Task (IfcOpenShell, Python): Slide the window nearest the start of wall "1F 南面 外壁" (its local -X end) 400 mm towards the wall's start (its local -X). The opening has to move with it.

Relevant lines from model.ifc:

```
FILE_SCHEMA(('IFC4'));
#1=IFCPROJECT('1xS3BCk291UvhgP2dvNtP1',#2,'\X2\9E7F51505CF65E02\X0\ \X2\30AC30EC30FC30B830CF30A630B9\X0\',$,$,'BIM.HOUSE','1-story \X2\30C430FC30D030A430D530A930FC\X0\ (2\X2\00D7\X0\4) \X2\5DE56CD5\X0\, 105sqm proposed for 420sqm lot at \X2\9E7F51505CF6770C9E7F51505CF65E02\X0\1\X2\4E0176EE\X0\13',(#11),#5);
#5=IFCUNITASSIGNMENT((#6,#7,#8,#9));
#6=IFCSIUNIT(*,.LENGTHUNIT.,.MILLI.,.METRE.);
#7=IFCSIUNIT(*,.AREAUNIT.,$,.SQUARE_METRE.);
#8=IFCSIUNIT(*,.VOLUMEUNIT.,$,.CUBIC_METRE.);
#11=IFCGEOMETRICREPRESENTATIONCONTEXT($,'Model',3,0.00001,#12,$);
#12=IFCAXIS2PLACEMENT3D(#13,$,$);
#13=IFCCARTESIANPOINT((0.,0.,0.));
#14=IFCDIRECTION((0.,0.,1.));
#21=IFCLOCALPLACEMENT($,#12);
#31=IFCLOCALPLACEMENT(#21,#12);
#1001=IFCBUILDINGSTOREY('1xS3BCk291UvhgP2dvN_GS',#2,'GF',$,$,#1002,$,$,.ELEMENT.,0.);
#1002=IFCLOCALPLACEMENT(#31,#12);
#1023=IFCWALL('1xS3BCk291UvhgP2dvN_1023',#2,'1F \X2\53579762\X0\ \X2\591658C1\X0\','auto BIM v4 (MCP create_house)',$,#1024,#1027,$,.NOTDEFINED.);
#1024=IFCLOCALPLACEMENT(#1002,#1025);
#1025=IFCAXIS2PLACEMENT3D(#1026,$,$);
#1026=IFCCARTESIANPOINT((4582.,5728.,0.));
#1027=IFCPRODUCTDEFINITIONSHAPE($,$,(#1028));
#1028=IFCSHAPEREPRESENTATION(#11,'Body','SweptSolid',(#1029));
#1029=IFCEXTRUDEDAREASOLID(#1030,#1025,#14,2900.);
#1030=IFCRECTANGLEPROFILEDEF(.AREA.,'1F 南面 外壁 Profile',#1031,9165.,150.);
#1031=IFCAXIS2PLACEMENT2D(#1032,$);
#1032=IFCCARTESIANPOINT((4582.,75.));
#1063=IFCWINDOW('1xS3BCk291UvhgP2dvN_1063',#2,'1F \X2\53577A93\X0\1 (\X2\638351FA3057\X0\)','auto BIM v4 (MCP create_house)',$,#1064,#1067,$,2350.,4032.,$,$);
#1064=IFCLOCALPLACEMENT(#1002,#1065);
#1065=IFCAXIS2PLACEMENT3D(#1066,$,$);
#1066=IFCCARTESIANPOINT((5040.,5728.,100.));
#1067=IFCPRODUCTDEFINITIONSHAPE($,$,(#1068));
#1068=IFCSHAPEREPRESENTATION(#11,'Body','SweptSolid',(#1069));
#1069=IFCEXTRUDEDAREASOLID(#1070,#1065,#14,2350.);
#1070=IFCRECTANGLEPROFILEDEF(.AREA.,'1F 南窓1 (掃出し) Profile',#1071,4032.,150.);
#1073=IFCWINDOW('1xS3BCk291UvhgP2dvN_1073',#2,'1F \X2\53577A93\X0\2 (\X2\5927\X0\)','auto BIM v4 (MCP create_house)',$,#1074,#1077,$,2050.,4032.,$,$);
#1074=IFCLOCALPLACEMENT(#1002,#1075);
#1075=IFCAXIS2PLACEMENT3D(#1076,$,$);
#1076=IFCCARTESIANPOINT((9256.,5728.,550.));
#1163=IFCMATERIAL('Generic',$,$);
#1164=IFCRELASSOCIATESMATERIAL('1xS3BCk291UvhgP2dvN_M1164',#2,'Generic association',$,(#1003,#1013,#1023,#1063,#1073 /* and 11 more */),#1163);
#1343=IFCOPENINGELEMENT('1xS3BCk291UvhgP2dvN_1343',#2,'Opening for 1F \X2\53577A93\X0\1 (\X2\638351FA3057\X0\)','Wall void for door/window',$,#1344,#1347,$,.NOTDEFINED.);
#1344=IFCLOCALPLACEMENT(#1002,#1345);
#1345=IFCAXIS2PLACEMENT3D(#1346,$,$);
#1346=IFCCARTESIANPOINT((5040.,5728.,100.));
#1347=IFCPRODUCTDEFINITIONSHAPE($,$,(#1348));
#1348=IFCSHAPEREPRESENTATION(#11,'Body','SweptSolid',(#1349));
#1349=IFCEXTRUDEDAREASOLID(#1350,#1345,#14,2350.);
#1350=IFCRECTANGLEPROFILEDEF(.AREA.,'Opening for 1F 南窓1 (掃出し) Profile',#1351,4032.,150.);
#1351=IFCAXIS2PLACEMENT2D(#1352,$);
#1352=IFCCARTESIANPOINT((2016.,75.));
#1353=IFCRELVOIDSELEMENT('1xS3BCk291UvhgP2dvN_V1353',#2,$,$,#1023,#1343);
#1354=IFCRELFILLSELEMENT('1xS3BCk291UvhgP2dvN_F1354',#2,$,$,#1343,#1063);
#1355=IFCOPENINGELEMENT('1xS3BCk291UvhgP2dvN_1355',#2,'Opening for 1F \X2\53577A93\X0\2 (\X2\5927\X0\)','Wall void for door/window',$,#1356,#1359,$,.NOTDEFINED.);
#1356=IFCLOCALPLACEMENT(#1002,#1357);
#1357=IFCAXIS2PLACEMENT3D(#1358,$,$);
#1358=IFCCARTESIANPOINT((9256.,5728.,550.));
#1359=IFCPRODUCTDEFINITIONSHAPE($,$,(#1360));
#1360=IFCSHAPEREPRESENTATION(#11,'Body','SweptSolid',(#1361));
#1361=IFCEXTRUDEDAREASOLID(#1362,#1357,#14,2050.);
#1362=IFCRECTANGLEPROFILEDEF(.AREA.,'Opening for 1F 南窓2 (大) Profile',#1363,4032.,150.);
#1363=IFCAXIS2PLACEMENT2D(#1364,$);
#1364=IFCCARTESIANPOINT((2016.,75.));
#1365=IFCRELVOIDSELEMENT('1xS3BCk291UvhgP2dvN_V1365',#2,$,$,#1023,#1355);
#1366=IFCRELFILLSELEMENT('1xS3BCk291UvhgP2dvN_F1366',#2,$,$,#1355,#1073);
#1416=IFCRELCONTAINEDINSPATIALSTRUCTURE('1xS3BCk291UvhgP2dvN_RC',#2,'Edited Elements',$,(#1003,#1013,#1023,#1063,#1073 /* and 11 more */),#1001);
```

```python
import ifcopenshell
import ifcopenshell.api.geometry
import ifcopenshell.util.placement

model = ifcopenshell.open("model.ifc")

window = model.by_id(1063)
opening = window.FillsVoids[0].RelatingOpeningElement
wall = opening.VoidsElements[0].RelatingBuildingElement

wall_matrix = ifcopenshell.util.placement.get_local_placement(wall.ObjectPlacement)
shift = wall_matrix[:3, 0] * -400.0
before = ifcopenshell.util.placement.get_local_placement(window.ObjectPlacement)[:3, 3].copy()

# The window is not placed relative to its opening, so move both.
for product in (opening, window):
    matrix = ifcopenshell.util.placement.get_local_placement(product.ObjectPlacement)
    matrix[:3, 3] += shift
    ifcopenshell.api.geometry.edit_object_placement(model, product=product, matrix=matrix, is_si=False)

after = ifcopenshell.util.placement.get_local_placement(window.ObjectPlacement)[:3, 3]
print("window moved by", (after - before).round(3) + 0.0)

model.write("model_edited.ifc")
```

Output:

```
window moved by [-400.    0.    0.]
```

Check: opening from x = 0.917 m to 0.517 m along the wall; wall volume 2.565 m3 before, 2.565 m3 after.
